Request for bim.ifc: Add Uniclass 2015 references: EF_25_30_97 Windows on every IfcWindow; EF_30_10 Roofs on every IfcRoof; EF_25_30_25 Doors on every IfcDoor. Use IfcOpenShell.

First a look at what the model holds.

```python
import ifcopenshell

model = ifcopenshell.open("bim.ifc")
print(model.schema)
print("classifications:", [c.Name for c in model.by_type("IfcClassification")])
for ifc_class in ("IfcDoor", "IfcRoof", "IfcStair", "IfcWall", "IfcWindow"):
    print(ifc_class, len(model.by_type(ifc_class)))
```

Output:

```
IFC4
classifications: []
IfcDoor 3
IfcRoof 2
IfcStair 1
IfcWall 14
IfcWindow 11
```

```python
import ifcopenshell
import ifcopenshell.api.classification

model = ifcopenshell.open("bim.ifc")

system = ifcopenshell.api.classification.add_classification(model, classification="Uniclass 2015")

codes = {
    "IfcWindow": ("EF_25_30_97", "Windows"),
    "IfcRoof": ("EF_30_10", "Roofs"),
    "IfcDoor": ("EF_25_30_25", "Doors"),
}
for ifc_class, (code, name) in codes.items():
    products = model.by_type(ifc_class)
    ifcopenshell.api.classification.add_reference(
        model, products=products, classification=system, identification=code, name=name
    )
    print(code, len(products))

model.write("bim_edited.ifc")
```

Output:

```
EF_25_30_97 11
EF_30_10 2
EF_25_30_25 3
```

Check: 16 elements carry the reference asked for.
